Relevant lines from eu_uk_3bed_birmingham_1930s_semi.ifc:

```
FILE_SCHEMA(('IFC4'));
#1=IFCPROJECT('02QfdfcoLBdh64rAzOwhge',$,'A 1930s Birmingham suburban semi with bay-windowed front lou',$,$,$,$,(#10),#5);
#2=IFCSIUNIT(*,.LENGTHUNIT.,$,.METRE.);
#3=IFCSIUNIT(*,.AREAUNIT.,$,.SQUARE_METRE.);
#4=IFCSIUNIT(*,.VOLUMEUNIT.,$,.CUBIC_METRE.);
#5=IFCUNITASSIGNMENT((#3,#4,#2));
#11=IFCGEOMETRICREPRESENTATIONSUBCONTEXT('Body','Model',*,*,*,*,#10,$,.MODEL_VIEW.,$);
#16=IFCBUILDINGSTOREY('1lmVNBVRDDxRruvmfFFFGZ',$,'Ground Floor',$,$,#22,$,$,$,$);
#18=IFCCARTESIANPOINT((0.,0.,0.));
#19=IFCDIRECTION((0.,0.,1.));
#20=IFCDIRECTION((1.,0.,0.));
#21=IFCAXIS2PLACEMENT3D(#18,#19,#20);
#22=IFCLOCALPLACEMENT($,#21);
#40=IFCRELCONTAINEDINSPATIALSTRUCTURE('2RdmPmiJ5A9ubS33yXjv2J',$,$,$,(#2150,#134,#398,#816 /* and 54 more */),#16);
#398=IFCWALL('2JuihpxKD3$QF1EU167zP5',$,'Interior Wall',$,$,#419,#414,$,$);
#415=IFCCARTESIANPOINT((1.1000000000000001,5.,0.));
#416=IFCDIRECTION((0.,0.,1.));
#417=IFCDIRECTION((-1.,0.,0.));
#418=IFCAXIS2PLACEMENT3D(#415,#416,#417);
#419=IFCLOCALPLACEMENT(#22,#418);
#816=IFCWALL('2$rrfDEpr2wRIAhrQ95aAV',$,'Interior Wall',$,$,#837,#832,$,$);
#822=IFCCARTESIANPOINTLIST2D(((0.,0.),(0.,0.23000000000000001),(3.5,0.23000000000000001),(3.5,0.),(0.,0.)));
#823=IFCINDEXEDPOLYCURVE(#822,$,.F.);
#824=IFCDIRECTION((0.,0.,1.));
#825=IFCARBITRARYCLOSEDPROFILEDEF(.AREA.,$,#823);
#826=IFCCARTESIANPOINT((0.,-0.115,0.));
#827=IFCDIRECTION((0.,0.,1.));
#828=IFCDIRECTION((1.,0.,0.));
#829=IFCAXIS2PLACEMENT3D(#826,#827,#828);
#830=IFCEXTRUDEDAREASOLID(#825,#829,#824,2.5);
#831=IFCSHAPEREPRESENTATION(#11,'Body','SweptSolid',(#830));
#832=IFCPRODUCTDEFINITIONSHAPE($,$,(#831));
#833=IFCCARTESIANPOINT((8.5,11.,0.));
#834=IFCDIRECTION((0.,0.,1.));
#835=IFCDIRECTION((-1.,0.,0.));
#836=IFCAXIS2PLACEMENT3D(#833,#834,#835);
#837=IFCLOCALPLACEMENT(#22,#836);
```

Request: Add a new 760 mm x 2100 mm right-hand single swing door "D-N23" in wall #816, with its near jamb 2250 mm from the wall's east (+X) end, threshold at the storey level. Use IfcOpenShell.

```python
import numpy as np
import ifcopenshell
import ifcopenshell.api.feature
import ifcopenshell.api.geometry
import ifcopenshell.api.root
import ifcopenshell.api.spatial
import ifcopenshell.geom
import ifcopenshell.util.element
import ifcopenshell.util.placement
import ifcopenshell.util.representation
import ifcopenshell.util.shape
import ifcopenshell.util.unit

model = ifcopenshell.open("eu_uk_3bed_birmingham_1930s_semi.ifc")
unit_scale = ifcopenshell.util.unit.calculate_unit_scale(model)
settings = ifcopenshell.geom.settings()


def volume(element):
    """Net volume in cubic metres, openings subtracted."""
    shape = ifcopenshell.geom.create_shape(settings, element)
    return ifcopenshell.util.shape.get_volume(shape.geometry)


wall = model.by_id(816)
storey = ifcopenshell.util.element.get_container(wall, ifc_class="IfcBuildingStorey")
context = ifcopenshell.util.representation.get_context(model, "Model", "Body", "MODEL_VIEW")
before = volume(wall)

width, height, from_end, sill = 0.76, 2.1, 2.25, 0.0  # metres

# The wall runs along its own X axis, and the end named is its -X end.
wall_shape = ifcopenshell.geom.create_shape(settings, wall)
x, y, z = ifcopenshell.util.shape.get_vertices(wall_shape.geometry).T
start = x.min() + from_end
face, thickness = float(y.min()), float(y.max() - y.min())
wall_matrix = ifcopenshell.util.placement.get_local_placement(wall.ObjectPlacement)
level = ifcopenshell.util.placement.get_local_placement(storey.ObjectPlacement)[2, 3]


def in_wall(x, y):
    """Placement at x, y metres in the wall's axes, at sill height."""
    matrix = wall_matrix.copy()
    matrix[:, 3] = wall_matrix @ np.array([x / unit_scale, y / unit_scale, 0.0, 1.0])
    matrix[2, 3] = level + sill / unit_scale
    return matrix


# Opening: a box that overshoots both wall faces by 50 mm.
opening = ifcopenshell.api.root.create_entity(model, ifc_class="IfcOpeningElement", predefined_type="OPENING")
box = ifcopenshell.api.geometry.add_wall_representation(
    model, context=context, length=width, height=height, thickness=thickness + 0.1
)
ifcopenshell.api.geometry.assign_representation(model, product=opening, representation=box)
ifcopenshell.api.geometry.edit_object_placement(model, product=opening, matrix=in_wall(start, face - 0.05), is_si=False)
ifcopenshell.api.feature.add_feature(model, feature=opening, element=wall)

door = ifcopenshell.api.root.create_entity(model, ifc_class="IfcDoor", name="D-N23", predefined_type="DOOR")
door.OverallWidth, door.OverallHeight = width / unit_scale, height / unit_scale
door.OperationType = "SINGLE_SWING_RIGHT"
body = ifcopenshell.api.geometry.add_door_representation(
    model,
    context=context,
    overall_width=door.OverallWidth,
    overall_height=door.OverallHeight,
    operation_type="SINGLE_SWING_RIGHT",
    lining_properties={"LiningDepth": thickness / unit_scale, "ThresholdDepth": thickness / unit_scale},
)
ifcopenshell.api.geometry.assign_representation(model, product=door, representation=body)
ifcopenshell.api.spatial.assign_container(model, products=[door], relating_structure=storey)
ifcopenshell.api.feature.add_filling(model, opening=opening, element=door)

# The lining spans the wall, so the door starts at the wall face.
ifcopenshell.api.geometry.edit_object_placement(model, product=door, matrix=in_wall(start, face), is_si=False)

after = volume(wall)

print(f"wall volume {before:.3f} -> {after:.3f} m3")

model.write("eu_uk_3bed_birmingham_1930s_semi-out.ifc")
```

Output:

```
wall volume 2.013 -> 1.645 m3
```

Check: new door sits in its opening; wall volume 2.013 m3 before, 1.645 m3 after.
